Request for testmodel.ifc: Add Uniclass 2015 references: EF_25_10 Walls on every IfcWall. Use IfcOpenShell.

First a look at what the model holds.

```python
import ifcopenshell

model = ifcopenshell.open("testmodel.ifc")
print(model.schema)
print("classifications:", [c.Name for c in model.by_type("IfcClassification")])
for ifc_class in ("IfcDoor", "IfcRoof", "IfcStair", "IfcWall", "IfcWindow"):
    print(ifc_class, len(model.by_type(ifc_class)))
```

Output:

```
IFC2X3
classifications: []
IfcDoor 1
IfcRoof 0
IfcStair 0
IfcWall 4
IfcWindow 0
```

```python
import ifcopenshell
import ifcopenshell.api.classification

model = ifcopenshell.open("testmodel.ifc")

# IFC2X3 requires Source and Edition and has no link from the project to the system.
system = model.create_entity("IfcClassification", Source="NBS", Edition="2015", Name="Uniclass 2015")

codes = {
    "IfcWall": ("EF_25_10", "Walls"),
}
for ifc_class, (code, name) in codes.items():
    products = model.by_type(ifc_class)
    ifcopenshell.api.classification.add_reference(
        model, products=products, classification=system, identification=code, name=name
    )
    print(code, len(products))

model.write("testmodel_edited.ifc")
```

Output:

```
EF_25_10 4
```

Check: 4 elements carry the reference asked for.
